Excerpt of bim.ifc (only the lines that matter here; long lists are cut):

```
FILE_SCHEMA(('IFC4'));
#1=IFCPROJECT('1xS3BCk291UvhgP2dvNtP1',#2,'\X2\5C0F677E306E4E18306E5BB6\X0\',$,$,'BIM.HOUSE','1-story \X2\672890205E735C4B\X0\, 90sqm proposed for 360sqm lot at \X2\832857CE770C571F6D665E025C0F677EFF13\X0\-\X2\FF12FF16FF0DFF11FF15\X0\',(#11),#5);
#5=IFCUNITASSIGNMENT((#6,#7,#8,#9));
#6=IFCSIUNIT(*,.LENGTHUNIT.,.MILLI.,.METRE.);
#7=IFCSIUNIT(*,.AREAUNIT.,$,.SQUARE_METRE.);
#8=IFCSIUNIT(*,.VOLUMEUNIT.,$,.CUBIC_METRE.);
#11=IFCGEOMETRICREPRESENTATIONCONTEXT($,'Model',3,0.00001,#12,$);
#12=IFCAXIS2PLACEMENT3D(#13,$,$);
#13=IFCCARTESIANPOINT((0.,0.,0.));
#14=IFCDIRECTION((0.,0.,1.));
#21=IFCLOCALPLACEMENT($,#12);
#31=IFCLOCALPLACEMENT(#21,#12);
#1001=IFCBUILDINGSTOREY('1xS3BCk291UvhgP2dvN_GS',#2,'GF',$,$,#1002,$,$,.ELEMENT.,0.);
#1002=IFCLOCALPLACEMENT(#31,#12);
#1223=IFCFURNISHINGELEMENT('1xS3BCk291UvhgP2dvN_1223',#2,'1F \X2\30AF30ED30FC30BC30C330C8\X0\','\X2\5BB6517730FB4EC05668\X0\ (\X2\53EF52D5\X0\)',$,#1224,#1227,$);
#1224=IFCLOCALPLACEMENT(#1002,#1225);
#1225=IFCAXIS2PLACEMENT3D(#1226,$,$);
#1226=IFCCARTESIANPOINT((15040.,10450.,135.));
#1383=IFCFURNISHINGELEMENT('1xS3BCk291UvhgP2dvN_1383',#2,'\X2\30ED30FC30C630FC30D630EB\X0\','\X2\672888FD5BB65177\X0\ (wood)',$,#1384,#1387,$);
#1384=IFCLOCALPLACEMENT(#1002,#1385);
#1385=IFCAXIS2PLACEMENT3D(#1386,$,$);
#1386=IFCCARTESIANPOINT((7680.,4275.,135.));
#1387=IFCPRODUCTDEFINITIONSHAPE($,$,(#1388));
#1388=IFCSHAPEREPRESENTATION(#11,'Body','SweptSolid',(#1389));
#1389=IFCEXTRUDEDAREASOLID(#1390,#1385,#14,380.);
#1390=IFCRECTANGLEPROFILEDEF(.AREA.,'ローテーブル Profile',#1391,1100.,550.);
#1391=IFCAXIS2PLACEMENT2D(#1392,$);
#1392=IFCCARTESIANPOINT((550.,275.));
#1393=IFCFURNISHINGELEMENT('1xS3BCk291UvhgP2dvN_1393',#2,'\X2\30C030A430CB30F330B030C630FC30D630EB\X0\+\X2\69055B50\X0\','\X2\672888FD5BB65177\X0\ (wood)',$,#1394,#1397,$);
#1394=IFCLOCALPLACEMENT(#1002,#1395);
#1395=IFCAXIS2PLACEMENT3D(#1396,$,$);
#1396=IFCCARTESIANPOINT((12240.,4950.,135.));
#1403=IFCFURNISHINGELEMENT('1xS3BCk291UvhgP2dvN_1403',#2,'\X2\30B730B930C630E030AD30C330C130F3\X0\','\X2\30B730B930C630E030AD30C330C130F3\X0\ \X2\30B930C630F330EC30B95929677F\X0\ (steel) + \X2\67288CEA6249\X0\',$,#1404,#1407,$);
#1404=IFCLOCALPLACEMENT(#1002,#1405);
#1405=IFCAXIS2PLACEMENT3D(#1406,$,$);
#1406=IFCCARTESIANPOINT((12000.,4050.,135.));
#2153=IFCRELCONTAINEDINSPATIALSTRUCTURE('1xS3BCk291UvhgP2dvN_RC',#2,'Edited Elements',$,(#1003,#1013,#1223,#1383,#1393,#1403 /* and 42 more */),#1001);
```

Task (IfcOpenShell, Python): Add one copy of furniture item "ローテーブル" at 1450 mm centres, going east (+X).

```python
import numpy as np
import ifcopenshell
import ifcopenshell.api.geometry
import ifcopenshell.api.root
import ifcopenshell.util.element
import ifcopenshell.util.placement

model = ifcopenshell.open("bim.ifc")


def reuse_history(source, copy):
    """copy_class also copies each property set's owner history, people and application; keep the originals."""
    for rel in copy.IsDefinedBy:
        if rel.is_a("IfcRelDefinesByProperties") and (history := rel.RelatingPropertyDefinition.OwnerHistory):
            rel.RelatingPropertyDefinition.OwnerHistory = source.OwnerHistory
            ifcopenshell.util.element.remove_deep2(model, history)


source = model.by_guid("1xS3BCk291UvhgP2dvN_1383")
base = ifcopenshell.util.placement.get_local_placement(source.ObjectPlacement)
step = np.array([1.0, 0.0, 0.0]) * 1450.0

for i in range(1, 2):
    copy = ifcopenshell.api.root.copy_class(model, product=source)
    copy.Representation = ifcopenshell.util.element.copy_deep(
        model, source.Representation, exclude=["IfcGeometricRepresentationContext", "IfcRepresentationMap"]
    )
    reuse_history(source, copy)
    matrix = base.copy()
    matrix[:3, 3] += i * step
    print("added at", matrix[:3, 3].round(3) + 0.0)
    ifcopenshell.api.geometry.edit_object_placement(model, product=copy, matrix=matrix, is_si=False)

model.write("bim_v2.ifc")
```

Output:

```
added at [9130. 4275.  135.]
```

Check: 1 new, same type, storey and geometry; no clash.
